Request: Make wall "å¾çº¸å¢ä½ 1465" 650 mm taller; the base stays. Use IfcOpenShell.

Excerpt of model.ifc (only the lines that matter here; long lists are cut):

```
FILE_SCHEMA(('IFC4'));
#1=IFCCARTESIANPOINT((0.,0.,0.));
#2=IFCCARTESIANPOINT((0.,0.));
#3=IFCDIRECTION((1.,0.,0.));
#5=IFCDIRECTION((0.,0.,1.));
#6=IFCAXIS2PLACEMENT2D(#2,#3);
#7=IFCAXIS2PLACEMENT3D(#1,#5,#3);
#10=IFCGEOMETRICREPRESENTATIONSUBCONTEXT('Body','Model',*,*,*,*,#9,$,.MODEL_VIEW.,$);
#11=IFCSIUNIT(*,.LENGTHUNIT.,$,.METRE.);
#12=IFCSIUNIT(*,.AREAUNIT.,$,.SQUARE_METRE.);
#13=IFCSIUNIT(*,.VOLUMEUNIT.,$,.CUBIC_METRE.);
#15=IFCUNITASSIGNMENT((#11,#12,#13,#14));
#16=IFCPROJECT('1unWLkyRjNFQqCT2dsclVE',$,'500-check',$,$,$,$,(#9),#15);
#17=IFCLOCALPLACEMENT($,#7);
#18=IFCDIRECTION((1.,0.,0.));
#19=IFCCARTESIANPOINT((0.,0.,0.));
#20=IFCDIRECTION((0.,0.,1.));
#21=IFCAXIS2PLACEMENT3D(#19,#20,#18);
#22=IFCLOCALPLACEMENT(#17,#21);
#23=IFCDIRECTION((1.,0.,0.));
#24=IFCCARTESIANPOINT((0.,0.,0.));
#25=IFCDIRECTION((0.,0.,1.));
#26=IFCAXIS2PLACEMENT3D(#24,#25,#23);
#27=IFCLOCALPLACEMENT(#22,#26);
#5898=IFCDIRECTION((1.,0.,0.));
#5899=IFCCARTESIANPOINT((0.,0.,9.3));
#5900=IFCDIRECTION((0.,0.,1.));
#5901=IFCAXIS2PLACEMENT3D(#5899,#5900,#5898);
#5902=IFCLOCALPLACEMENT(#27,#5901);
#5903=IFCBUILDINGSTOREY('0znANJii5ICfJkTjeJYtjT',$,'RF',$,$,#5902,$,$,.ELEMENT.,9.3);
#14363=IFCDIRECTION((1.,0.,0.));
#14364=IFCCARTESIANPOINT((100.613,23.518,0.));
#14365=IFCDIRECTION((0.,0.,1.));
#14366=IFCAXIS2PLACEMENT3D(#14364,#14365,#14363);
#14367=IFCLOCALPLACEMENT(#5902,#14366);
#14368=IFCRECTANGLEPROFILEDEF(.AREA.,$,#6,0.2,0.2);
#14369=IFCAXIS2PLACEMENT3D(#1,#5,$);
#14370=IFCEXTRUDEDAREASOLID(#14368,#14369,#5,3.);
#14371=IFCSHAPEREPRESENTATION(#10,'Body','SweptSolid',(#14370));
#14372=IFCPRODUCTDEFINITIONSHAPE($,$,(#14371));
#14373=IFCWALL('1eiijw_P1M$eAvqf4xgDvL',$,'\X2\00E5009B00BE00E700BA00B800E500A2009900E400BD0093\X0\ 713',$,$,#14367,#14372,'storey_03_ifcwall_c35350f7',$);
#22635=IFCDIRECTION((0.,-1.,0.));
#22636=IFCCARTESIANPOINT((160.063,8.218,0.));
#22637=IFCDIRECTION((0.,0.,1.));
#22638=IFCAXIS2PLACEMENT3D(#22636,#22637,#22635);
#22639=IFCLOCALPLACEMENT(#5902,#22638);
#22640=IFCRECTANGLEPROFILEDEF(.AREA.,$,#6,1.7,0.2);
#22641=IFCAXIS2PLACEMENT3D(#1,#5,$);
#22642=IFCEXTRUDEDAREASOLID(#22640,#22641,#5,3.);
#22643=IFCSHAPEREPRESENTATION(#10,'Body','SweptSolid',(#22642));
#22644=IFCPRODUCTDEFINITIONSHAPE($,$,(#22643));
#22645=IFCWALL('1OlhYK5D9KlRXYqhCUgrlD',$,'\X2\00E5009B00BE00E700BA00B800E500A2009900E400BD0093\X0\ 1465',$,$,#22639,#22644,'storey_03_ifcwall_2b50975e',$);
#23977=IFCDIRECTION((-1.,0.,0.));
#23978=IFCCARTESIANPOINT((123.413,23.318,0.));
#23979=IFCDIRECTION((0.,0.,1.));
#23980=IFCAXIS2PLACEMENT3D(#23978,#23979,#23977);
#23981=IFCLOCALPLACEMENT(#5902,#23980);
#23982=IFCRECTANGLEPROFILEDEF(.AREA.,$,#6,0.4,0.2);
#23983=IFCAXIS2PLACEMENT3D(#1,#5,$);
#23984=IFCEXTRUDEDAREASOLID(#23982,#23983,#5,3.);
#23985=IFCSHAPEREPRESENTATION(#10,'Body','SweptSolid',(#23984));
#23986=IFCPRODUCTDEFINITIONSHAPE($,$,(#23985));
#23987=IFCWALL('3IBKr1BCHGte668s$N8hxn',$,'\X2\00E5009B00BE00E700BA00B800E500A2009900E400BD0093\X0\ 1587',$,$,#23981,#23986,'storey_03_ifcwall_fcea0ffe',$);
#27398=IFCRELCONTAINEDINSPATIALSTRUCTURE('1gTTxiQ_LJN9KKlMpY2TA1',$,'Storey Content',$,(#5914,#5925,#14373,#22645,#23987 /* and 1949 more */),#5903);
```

```python
import ifcopenshell
import ifcopenshell.geom
import ifcopenshell.util.representation
import ifcopenshell.util.shape
import ifcopenshell.util.unit

model = ifcopenshell.open("model.ifc")
unit_scale = ifcopenshell.util.unit.calculate_unit_scale(model)
settings = ifcopenshell.geom.settings()


def volume(element):
    """Net volume in cubic metres, openings subtracted."""
    shape = ifcopenshell.geom.create_shape(settings, element)
    return ifcopenshell.util.shape.get_volume(shape.geometry)


wall = model.by_guid("1OlhYK5D9KlRXYqhCUgrlD")
before = volume(wall)

body = ifcopenshell.util.representation.get_representation(wall, "Model", "Body")
solid = body.Items[0]
old_height = solid.Depth
solid.Depth += 0.65 / unit_scale
after = volume(wall)

print(f"height {old_height:g} -> {solid.Depth:g}, volume {before:.3f} -> {after:.3f} m3")

model.write("model-out.ifc")
```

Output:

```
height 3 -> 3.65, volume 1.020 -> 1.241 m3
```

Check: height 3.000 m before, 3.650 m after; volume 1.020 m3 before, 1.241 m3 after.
